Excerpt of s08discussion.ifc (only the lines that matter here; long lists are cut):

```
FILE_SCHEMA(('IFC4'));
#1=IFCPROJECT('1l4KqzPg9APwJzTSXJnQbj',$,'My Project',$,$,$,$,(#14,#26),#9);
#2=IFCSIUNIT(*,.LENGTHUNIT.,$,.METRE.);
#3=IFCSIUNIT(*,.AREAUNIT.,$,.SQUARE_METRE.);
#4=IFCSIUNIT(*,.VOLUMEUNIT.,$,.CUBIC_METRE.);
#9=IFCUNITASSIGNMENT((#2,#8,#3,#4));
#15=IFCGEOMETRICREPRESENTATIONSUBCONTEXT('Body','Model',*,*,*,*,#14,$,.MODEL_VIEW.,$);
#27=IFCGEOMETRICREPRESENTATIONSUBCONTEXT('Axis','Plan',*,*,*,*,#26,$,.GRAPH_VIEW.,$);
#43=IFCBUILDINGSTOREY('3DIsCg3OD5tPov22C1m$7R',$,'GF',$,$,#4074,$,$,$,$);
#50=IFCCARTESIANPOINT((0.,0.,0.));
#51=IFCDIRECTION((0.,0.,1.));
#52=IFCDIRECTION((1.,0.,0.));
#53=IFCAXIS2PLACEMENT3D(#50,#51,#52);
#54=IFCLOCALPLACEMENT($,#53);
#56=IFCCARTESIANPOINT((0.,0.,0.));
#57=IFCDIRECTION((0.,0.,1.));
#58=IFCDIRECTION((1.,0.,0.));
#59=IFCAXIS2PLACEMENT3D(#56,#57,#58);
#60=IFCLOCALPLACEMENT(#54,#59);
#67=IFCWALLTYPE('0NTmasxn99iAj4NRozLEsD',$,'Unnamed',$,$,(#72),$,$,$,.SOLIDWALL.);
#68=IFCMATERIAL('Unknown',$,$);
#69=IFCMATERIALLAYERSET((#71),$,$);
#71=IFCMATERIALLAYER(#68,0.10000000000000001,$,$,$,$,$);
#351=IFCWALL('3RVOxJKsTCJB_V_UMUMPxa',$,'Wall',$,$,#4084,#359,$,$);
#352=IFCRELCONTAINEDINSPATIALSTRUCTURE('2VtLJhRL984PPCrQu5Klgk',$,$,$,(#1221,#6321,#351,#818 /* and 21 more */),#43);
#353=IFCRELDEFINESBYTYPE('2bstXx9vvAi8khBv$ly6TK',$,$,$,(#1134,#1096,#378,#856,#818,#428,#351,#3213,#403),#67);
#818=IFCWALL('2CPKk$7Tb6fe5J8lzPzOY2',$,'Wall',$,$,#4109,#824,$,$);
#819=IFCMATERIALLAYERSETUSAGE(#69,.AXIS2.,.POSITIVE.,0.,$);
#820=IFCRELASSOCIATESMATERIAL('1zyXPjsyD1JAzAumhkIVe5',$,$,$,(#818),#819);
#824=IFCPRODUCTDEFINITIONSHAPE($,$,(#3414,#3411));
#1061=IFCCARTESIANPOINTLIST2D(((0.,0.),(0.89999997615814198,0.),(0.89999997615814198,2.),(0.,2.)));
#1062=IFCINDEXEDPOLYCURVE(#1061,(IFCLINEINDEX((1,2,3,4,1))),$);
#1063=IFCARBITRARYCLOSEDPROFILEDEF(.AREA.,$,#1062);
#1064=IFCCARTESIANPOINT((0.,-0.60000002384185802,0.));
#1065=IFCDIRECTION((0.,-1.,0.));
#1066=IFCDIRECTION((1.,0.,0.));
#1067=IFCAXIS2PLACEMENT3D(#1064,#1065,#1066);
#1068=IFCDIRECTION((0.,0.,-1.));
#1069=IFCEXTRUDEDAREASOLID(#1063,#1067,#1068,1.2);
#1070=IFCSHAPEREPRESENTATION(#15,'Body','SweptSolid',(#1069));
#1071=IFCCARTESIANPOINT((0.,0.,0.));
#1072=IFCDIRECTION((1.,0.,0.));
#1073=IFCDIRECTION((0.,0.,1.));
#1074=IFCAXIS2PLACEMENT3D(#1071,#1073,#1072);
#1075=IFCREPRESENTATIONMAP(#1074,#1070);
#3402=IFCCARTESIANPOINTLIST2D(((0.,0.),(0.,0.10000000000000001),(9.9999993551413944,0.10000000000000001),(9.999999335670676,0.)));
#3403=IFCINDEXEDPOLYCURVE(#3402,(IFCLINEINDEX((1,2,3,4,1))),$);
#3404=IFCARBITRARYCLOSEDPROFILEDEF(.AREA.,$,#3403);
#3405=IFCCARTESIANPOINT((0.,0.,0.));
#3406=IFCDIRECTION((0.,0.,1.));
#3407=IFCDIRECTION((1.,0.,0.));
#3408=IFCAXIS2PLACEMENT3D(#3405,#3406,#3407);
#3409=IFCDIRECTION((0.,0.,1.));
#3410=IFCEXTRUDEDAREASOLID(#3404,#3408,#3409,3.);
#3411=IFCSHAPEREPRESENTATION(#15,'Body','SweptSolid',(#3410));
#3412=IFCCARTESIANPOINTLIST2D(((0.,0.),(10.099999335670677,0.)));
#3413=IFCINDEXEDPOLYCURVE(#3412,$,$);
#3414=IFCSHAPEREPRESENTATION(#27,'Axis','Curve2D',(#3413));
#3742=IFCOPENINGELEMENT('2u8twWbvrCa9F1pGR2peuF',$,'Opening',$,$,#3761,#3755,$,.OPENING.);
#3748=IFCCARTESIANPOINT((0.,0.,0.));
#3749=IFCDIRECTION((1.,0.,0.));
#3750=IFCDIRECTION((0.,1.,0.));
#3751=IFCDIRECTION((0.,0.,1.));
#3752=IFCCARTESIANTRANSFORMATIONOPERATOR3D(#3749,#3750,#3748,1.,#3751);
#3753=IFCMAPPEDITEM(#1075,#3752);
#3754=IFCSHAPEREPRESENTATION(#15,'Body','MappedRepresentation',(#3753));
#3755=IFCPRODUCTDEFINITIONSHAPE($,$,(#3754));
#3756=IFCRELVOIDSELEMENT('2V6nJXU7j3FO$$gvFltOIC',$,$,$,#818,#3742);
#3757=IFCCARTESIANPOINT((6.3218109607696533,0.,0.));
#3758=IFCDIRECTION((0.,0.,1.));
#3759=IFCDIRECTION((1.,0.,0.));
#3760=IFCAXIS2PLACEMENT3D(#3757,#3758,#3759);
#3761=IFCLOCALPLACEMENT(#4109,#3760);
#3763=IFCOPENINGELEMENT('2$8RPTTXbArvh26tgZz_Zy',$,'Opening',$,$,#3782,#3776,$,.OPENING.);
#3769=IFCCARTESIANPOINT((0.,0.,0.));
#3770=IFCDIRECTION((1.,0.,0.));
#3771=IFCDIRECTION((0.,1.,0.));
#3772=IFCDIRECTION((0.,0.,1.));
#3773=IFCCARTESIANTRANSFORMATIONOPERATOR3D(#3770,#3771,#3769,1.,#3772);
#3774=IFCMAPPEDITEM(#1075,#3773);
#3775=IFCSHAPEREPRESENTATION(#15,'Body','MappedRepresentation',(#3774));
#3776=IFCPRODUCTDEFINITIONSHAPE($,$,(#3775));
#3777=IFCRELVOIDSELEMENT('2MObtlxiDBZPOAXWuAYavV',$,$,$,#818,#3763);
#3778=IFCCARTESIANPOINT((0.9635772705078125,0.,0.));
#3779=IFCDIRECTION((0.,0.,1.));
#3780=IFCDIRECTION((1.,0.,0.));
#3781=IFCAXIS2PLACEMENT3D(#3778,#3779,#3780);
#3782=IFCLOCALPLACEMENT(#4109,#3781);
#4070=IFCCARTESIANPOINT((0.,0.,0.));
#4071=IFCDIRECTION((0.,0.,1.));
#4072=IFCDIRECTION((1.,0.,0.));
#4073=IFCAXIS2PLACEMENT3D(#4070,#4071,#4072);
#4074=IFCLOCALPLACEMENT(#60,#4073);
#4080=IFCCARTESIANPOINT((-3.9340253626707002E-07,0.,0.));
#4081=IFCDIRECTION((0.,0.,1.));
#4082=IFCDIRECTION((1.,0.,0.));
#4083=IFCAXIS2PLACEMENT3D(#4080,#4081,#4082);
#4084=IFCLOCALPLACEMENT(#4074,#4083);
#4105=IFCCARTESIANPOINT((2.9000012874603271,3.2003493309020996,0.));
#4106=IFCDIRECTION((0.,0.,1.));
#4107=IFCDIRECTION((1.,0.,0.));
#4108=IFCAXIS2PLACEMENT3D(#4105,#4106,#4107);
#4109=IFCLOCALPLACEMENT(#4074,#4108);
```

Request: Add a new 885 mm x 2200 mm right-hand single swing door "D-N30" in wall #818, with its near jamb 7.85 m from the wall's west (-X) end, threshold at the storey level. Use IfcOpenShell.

```python
import numpy as np
import ifcopenshell
import ifcopenshell.api.feature
import ifcopenshell.api.geometry
import ifcopenshell.api.root
import ifcopenshell.api.spatial
import ifcopenshell.geom
import ifcopenshell.util.element
import ifcopenshell.util.placement
import ifcopenshell.util.representation
import ifcopenshell.util.shape
import ifcopenshell.util.unit

model = ifcopenshell.open("s08discussion.ifc")
unit_scale = ifcopenshell.util.unit.calculate_unit_scale(model)
settings = ifcopenshell.geom.settings()


def volume(element):
    """Net volume in cubic metres, openings subtracted."""
    shape = ifcopenshell.geom.create_shape(settings, element)
    return ifcopenshell.util.shape.get_volume(shape.geometry)


wall = model.by_guid("2CPKk$7Tb6fe5J8lzPzOY2")
storey = ifcopenshell.util.element.get_container(wall, ifc_class="IfcBuildingStorey")
context = ifcopenshell.util.representation.get_context(model, "Model", "Body", "MODEL_VIEW")
before = volume(wall)

width, height, from_end, sill = 0.885, 2.2, 7.85, 0.0  # metres

# The wall runs along its own X axis, and the end named is its -X end.
wall_shape = ifcopenshell.geom.create_shape(settings, wall)
x, y, z = ifcopenshell.util.shape.get_vertices(wall_shape.geometry).T
start = x.min() + from_end
face, thickness = float(y.min()), float(y.max() - y.min())
wall_matrix = ifcopenshell.util.placement.get_local_placement(wall.ObjectPlacement)
level = ifcopenshell.util.placement.get_local_placement(storey.ObjectPlacement)[2, 3]


def in_wall(x, y):
    """Placement at x, y metres in the wall's axes, at sill height."""
    matrix = wall_matrix.copy()
    matrix[:, 3] = wall_matrix @ np.array([x / unit_scale, y / unit_scale, 0.0, 1.0])
    matrix[2, 3] = level + sill / unit_scale
    return matrix


# Opening: a box that overshoots both wall faces by 50 mm.
opening = ifcopenshell.api.root.create_entity(model, ifc_class="IfcOpeningElement", predefined_type="OPENING")
box = ifcopenshell.api.geometry.add_wall_representation(
    model, context=context, length=width, height=height, thickness=thickness + 0.1
)
ifcopenshell.api.geometry.assign_representation(model, product=opening, representation=box)
ifcopenshell.api.geometry.edit_object_placement(model, product=opening, matrix=in_wall(start, face - 0.05), is_si=False)
ifcopenshell.api.feature.add_feature(model, feature=opening, element=wall)

door = ifcopenshell.api.root.create_entity(model, ifc_class="IfcDoor", name="D-N30", predefined_type="DOOR")
door.OverallWidth, door.OverallHeight = width / unit_scale, height / unit_scale
door.OperationType = "SINGLE_SWING_RIGHT"
body = ifcopenshell.api.geometry.add_door_representation(
    model,
    context=context,
    overall_width=door.OverallWidth,
    overall_height=door.OverallHeight,
    operation_type="SINGLE_SWING_RIGHT",
    lining_properties={"LiningDepth": thickness / unit_scale, "ThresholdDepth": thickness / unit_scale},
)
ifcopenshell.api.geometry.assign_representation(model, product=door, representation=body)
ifcopenshell.api.spatial.assign_container(model, products=[door], relating_structure=storey)
ifcopenshell.api.feature.add_filling(model, opening=opening, element=door)

# The lining spans the wall, so the door starts at the wall face.
ifcopenshell.api.geometry.edit_object_placement(model, product=door, matrix=in_wall(start, face), is_si=False)

after = volume(wall)

print(f"wall volume {before:.3f} -> {after:.3f} m3")

model.write("s08discussion_updated.ifc")
```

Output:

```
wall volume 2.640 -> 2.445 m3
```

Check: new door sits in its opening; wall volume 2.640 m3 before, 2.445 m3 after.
